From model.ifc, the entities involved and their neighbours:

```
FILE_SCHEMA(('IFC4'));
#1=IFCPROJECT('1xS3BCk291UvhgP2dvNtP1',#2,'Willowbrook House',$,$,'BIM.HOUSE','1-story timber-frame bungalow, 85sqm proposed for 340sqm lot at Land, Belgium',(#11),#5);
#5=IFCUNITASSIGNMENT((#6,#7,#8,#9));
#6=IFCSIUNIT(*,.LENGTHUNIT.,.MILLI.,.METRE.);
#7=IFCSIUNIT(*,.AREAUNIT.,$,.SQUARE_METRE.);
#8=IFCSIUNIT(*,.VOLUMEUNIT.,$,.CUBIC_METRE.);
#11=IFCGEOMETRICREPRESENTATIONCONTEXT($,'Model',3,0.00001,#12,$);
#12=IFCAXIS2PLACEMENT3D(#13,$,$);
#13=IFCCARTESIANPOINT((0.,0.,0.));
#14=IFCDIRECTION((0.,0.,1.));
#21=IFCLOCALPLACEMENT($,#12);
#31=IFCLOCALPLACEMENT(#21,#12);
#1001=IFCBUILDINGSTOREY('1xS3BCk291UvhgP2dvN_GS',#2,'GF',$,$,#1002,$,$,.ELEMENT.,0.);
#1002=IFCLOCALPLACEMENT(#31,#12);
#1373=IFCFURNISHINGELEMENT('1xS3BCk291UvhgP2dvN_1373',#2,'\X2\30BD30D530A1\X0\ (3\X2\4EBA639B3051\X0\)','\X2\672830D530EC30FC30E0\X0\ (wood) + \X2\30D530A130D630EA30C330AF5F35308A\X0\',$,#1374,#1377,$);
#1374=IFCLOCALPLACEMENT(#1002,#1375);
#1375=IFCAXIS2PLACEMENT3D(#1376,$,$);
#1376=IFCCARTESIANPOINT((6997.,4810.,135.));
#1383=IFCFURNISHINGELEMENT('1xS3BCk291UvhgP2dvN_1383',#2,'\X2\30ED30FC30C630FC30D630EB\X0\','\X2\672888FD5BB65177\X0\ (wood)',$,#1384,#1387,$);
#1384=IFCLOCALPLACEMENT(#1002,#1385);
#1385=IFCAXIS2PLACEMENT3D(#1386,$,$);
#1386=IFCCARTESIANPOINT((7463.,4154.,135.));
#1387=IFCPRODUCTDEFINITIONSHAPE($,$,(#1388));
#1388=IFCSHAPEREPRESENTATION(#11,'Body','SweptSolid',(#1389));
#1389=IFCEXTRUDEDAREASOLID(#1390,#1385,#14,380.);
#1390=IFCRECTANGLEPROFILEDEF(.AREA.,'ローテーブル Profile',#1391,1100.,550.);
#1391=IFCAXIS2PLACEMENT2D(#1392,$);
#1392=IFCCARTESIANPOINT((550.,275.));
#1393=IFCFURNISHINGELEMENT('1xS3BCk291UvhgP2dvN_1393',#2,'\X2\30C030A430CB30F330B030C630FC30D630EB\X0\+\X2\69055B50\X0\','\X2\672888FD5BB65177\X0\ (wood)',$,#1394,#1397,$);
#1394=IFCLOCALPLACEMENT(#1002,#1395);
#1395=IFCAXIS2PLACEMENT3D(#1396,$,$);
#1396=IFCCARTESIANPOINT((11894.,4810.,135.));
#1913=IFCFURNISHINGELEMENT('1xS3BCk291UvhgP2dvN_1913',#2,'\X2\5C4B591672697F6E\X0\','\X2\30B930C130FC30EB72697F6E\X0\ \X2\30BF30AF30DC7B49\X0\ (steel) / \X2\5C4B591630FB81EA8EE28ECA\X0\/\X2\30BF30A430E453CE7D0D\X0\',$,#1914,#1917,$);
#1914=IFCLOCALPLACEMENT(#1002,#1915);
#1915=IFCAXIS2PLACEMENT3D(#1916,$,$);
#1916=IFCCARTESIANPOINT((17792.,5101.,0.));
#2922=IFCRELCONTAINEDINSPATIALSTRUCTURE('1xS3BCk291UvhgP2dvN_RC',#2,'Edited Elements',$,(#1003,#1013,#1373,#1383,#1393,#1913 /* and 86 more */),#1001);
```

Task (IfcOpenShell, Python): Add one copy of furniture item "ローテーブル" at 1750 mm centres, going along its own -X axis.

```python
import ifcopenshell
import ifcopenshell.api.geometry
import ifcopenshell.api.root
import ifcopenshell.util.element
import ifcopenshell.util.placement
import ifcopenshell.util.unit

model = ifcopenshell.open("model.ifc")
unit_scale = ifcopenshell.util.unit.calculate_unit_scale(model)


def reuse_history(source, copy):
    """copy_class also copies each property set's owner history, people and application; keep the originals."""
    for rel in copy.IsDefinedBy:
        if rel.is_a("IfcRelDefinesByProperties") and (history := rel.RelatingPropertyDefinition.OwnerHistory):
            rel.RelatingPropertyDefinition.OwnerHistory = source.OwnerHistory
            ifcopenshell.util.element.remove_deep2(model, history)


source = model.by_guid("1xS3BCk291UvhgP2dvN_1383")
base = ifcopenshell.util.placement.get_local_placement(source.ObjectPlacement)
step = -base[:3, 0] * 1.75 / unit_scale

for i in range(1, 2):
    copy = ifcopenshell.api.root.copy_class(model, product=source)
    copy.Representation = ifcopenshell.util.element.copy_deep(
        model, source.Representation, exclude=["IfcGeometricRepresentationContext", "IfcRepresentationMap"]
    )
    reuse_history(source, copy)
    matrix = base.copy()
    matrix[:3, 3] += i * step
    print("added at", matrix[:3, 3].round(3) + 0.0)
    ifcopenshell.api.geometry.edit_object_placement(model, product=copy, matrix=matrix, is_si=False)

model.write("model_v2.ifc")
```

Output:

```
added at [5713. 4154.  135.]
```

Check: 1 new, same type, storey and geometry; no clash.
